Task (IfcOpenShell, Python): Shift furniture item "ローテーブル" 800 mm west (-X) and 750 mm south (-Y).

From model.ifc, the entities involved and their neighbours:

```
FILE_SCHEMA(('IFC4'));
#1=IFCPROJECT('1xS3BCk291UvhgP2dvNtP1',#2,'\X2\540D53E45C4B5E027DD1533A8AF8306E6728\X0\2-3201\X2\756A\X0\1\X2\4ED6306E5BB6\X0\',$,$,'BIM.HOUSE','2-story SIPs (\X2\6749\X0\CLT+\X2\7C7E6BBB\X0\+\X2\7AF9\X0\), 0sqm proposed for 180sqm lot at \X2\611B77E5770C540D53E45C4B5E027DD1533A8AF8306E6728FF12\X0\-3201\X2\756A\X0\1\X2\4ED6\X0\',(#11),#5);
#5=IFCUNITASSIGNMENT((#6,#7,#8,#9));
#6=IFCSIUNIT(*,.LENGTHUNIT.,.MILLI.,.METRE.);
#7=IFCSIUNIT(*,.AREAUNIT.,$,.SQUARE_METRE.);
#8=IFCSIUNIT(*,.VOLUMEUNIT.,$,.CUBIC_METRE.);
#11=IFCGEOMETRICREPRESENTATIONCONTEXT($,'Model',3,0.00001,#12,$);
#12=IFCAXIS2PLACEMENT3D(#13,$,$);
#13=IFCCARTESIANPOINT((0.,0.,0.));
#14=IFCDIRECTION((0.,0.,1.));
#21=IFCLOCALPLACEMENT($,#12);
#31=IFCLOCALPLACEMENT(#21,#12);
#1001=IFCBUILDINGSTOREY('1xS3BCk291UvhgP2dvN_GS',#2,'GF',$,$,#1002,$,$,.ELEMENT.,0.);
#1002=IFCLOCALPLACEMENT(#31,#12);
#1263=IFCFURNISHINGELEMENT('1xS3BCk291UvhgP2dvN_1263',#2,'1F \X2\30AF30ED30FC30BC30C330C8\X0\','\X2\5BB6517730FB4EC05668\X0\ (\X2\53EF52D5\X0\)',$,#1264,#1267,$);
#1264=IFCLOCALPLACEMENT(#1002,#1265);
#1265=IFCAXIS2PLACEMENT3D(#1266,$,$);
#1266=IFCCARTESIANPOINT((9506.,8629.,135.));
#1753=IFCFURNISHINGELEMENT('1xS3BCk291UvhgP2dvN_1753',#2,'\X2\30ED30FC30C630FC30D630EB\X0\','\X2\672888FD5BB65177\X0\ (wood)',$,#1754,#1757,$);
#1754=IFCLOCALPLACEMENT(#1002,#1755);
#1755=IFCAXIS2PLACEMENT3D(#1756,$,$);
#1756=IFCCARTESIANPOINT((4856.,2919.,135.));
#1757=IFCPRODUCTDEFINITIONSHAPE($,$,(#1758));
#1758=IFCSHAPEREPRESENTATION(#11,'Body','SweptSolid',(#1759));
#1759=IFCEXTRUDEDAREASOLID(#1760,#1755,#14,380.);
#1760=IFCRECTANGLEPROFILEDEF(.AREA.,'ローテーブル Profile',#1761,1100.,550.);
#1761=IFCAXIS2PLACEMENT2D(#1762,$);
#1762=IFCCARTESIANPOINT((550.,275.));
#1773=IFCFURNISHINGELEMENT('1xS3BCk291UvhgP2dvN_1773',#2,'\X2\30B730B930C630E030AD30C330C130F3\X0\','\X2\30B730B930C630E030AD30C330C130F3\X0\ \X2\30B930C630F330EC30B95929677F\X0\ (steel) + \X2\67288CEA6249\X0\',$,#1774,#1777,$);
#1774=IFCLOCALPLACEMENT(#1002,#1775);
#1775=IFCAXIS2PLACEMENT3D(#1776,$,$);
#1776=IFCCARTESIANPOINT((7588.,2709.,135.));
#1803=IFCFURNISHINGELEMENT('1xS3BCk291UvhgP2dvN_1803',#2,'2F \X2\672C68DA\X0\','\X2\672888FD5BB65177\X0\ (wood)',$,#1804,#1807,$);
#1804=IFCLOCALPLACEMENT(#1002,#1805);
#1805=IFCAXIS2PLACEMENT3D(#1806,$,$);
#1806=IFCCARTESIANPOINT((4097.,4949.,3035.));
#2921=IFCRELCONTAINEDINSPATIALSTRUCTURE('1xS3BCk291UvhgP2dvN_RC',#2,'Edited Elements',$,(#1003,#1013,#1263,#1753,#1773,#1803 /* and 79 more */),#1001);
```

```python
import ifcopenshell
import ifcopenshell.api.geometry
import ifcopenshell.util.placement
import ifcopenshell.util.unit

model = ifcopenshell.open("model.ifc")
unit_scale = ifcopenshell.util.unit.calculate_unit_scale(model)

item = model.by_guid("1xS3BCk291UvhgP2dvN_1753")
matrix = ifcopenshell.util.placement.get_local_placement(item.ObjectPlacement)
matrix[0, 3] -= 0.8 / unit_scale
matrix[1, 3] -= 0.75 / unit_scale
ifcopenshell.api.geometry.edit_object_placement(model, product=item, matrix=matrix, is_si=False)

print(ifcopenshell.util.placement.get_local_placement(item.ObjectPlacement).round(3) + 0.0)

model.write("model-out.ifc")
```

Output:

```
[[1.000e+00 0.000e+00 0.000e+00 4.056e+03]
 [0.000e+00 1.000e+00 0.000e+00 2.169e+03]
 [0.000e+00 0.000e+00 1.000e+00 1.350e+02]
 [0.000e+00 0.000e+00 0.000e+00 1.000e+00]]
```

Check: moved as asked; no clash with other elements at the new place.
